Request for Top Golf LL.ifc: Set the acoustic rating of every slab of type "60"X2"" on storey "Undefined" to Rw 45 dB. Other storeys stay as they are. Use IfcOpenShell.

First a look at what the model holds.

```python
import ifcopenshell
import ifcopenshell.util.element

model = ifcopenshell.open("Top Golf LL.ifc")
print(model.schema)
storey = next(s for s in model.by_type("IfcBuildingStorey") if s.Name == "Undefined")
slabs = [e for e in ifcopenshell.util.element.get_decomposition(storey) if e.is_a("IfcSlab")]
seen = {}
for e in slabs:
    element_type = ifcopenshell.util.element.get_type(e)
    key = (element_type.Name if element_type != e and element_type else None, ifcopenshell.util.element.get_pset(e, "Pset_SlabCommon", "AcousticRating"))
    seen[key] = seen.get(key, 0) + 1
for (name, value), count in sorted(seen.items(), key=str):
    print(count, "x", name, "|", value)
```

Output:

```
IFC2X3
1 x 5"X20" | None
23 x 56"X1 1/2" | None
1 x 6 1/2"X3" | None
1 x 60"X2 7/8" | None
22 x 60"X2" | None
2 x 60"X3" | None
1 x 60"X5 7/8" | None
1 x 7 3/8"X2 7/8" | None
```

```python
import ifcopenshell
import ifcopenshell.api.pset
import ifcopenshell.util.element

model = ifcopenshell.open("Top Golf LL.ifc")

storey = next(s for s in model.by_type("IfcBuildingStorey") if s.Name == "Undefined")
slabs = [e for e in ifcopenshell.util.element.get_decomposition(storey) if e.is_a("IfcSlab")]

count = 0
for e in slabs:
    element_type = ifcopenshell.util.element.get_type(e)
    if element_type in (None, e) or element_type.Name != '60"X2"':
        continue
    found = ifcopenshell.util.element.get_pset(e, "Pset_SlabCommon", should_inherit=False)
    if found:
        pset = model.by_id(found["id"])
        if len(ifcopenshell.util.element.get_elements_by_pset(pset)) > 1:
            pset = ifcopenshell.api.pset.unshare_pset(model, products=[e], pset=pset)[0]
    else:
        pset = ifcopenshell.api.pset.add_pset(model, product=e, name="Pset_SlabCommon")
    ifcopenshell.api.pset.edit_pset(model, pset=pset, properties={"AcousticRating": "Rw 45 dB"})
    count += 1

print(count, "slabs updated")

model.write("Top Golf LL_v2.ifc")
```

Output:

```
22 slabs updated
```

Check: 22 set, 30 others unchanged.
